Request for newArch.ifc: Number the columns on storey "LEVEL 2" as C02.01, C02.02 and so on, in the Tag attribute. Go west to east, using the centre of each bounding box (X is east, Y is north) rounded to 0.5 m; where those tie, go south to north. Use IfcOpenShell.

First a look at what the model holds.

```python
import ifcopenshell
import ifcopenshell.util.element
import ifcopenshell.util.placement

model = ifcopenshell.open("newArch.ifc")
print(model.schema)
storey = next(s for s in model.by_type("IfcBuildingStorey") if s.Name == "LEVEL 2")
columns = [e for e in ifcopenshell.util.element.get_decomposition(storey) if e.is_a("IfcColumn")]
for e in sorted(columns, key=lambda e: e.id()):
    origin = ifcopenshell.util.placement.get_local_placement(e.ObjectPlacement)[:3, 3]
    print(e.id(), e.Tag, e.Name, origin.round(2) + 0.0, sep=" | ")
```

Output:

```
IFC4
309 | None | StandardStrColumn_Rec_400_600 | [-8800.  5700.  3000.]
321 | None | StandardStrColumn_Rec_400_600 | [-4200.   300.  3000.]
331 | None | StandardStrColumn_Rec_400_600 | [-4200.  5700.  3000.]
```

```python
import ifcopenshell
import ifcopenshell.geom
import ifcopenshell.util.element
import ifcopenshell.util.shape

model = ifcopenshell.open("newArch.ifc")
settings = ifcopenshell.geom.settings()
settings.set("use-world-coords", True)


def centre(element):
    shape = ifcopenshell.geom.create_shape(settings, element)
    return ifcopenshell.util.shape.get_bbox_centroid(shape.geometry)


storey = next(s for s in model.by_type("IfcBuildingStorey") if s.Name == "LEVEL 2")
columns = [e for e in ifcopenshell.util.element.get_decomposition(storey) if e.is_a("IfcColumn")]

# Insertion points can sit at a corner or the storey origin, so sort by the geometry (in metres).
centres = {e: centre(e) for e in columns}
columns.sort(key=lambda e: (round(centres[e][0] / 0.5), centres[e][1]))

for i, e in enumerate(columns, start=1):
    number = f"C02.{i:02d}"
    e.Tag = number
    print(e.id(), number)

model.write("newArch_v2.ifc")
```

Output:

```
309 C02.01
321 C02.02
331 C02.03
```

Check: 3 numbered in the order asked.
